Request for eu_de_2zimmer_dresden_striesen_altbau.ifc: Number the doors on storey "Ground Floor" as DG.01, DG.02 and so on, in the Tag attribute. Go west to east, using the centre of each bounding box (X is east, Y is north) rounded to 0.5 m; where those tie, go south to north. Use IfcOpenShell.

First a look at what the model holds.

```python
import ifcopenshell
import ifcopenshell.util.element
import ifcopenshell.util.placement

model = ifcopenshell.open("eu_de_2zimmer_dresden_striesen_altbau.ifc")
print(model.schema)
storey = next(s for s in model.by_type("IfcBuildingStorey") if s.Name == "Ground Floor")
doors = [e for e in ifcopenshell.util.element.get_decomposition(storey) if e.is_a("IfcDoor")]
for e in sorted(doors, key=lambda e: e.id()):
    origin = ifcopenshell.util.placement.get_local_placement(e.ObjectPlacement)[:3, 3]
    print(e.id(), e.Tag, e.Name, origin.round(2) + 0.0, sep=" | ")
```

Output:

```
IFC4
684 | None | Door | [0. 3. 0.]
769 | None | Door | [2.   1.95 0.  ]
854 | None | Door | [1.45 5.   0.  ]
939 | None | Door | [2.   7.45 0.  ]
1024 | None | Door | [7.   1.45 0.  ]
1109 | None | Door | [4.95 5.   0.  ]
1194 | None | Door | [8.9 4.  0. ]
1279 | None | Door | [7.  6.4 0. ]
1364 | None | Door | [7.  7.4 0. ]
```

```python
import ifcopenshell
import ifcopenshell.geom
import ifcopenshell.util.element
import ifcopenshell.util.shape

model = ifcopenshell.open("eu_de_2zimmer_dresden_striesen_altbau.ifc")
settings = ifcopenshell.geom.settings()
settings.set("use-world-coords", True)


def centre(element):
    shape = ifcopenshell.geom.create_shape(settings, element)
    return ifcopenshell.util.shape.get_bbox_centroid(shape.geometry)


storey = next(s for s in model.by_type("IfcBuildingStorey") if s.Name == "Ground Floor")
doors = [e for e in ifcopenshell.util.element.get_decomposition(storey) if e.is_a("IfcDoor")]

# Insertion points can sit at a corner or the storey origin, so sort by the geometry (in metres).
centres = {e: centre(e) for e in doors}
doors.sort(key=lambda e: (round(centres[e][0] / 0.5), centres[e][1]))

for i, e in enumerate(doors, start=1):
    number = f"DG.{i:02d}"
    e.Tag = number
    print(e.id(), number)

model.write("eu_de_2zimmer_dresden_striesen_altbau_updated.ifc")
```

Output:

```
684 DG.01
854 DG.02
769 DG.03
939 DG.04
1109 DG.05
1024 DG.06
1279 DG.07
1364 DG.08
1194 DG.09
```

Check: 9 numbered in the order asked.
